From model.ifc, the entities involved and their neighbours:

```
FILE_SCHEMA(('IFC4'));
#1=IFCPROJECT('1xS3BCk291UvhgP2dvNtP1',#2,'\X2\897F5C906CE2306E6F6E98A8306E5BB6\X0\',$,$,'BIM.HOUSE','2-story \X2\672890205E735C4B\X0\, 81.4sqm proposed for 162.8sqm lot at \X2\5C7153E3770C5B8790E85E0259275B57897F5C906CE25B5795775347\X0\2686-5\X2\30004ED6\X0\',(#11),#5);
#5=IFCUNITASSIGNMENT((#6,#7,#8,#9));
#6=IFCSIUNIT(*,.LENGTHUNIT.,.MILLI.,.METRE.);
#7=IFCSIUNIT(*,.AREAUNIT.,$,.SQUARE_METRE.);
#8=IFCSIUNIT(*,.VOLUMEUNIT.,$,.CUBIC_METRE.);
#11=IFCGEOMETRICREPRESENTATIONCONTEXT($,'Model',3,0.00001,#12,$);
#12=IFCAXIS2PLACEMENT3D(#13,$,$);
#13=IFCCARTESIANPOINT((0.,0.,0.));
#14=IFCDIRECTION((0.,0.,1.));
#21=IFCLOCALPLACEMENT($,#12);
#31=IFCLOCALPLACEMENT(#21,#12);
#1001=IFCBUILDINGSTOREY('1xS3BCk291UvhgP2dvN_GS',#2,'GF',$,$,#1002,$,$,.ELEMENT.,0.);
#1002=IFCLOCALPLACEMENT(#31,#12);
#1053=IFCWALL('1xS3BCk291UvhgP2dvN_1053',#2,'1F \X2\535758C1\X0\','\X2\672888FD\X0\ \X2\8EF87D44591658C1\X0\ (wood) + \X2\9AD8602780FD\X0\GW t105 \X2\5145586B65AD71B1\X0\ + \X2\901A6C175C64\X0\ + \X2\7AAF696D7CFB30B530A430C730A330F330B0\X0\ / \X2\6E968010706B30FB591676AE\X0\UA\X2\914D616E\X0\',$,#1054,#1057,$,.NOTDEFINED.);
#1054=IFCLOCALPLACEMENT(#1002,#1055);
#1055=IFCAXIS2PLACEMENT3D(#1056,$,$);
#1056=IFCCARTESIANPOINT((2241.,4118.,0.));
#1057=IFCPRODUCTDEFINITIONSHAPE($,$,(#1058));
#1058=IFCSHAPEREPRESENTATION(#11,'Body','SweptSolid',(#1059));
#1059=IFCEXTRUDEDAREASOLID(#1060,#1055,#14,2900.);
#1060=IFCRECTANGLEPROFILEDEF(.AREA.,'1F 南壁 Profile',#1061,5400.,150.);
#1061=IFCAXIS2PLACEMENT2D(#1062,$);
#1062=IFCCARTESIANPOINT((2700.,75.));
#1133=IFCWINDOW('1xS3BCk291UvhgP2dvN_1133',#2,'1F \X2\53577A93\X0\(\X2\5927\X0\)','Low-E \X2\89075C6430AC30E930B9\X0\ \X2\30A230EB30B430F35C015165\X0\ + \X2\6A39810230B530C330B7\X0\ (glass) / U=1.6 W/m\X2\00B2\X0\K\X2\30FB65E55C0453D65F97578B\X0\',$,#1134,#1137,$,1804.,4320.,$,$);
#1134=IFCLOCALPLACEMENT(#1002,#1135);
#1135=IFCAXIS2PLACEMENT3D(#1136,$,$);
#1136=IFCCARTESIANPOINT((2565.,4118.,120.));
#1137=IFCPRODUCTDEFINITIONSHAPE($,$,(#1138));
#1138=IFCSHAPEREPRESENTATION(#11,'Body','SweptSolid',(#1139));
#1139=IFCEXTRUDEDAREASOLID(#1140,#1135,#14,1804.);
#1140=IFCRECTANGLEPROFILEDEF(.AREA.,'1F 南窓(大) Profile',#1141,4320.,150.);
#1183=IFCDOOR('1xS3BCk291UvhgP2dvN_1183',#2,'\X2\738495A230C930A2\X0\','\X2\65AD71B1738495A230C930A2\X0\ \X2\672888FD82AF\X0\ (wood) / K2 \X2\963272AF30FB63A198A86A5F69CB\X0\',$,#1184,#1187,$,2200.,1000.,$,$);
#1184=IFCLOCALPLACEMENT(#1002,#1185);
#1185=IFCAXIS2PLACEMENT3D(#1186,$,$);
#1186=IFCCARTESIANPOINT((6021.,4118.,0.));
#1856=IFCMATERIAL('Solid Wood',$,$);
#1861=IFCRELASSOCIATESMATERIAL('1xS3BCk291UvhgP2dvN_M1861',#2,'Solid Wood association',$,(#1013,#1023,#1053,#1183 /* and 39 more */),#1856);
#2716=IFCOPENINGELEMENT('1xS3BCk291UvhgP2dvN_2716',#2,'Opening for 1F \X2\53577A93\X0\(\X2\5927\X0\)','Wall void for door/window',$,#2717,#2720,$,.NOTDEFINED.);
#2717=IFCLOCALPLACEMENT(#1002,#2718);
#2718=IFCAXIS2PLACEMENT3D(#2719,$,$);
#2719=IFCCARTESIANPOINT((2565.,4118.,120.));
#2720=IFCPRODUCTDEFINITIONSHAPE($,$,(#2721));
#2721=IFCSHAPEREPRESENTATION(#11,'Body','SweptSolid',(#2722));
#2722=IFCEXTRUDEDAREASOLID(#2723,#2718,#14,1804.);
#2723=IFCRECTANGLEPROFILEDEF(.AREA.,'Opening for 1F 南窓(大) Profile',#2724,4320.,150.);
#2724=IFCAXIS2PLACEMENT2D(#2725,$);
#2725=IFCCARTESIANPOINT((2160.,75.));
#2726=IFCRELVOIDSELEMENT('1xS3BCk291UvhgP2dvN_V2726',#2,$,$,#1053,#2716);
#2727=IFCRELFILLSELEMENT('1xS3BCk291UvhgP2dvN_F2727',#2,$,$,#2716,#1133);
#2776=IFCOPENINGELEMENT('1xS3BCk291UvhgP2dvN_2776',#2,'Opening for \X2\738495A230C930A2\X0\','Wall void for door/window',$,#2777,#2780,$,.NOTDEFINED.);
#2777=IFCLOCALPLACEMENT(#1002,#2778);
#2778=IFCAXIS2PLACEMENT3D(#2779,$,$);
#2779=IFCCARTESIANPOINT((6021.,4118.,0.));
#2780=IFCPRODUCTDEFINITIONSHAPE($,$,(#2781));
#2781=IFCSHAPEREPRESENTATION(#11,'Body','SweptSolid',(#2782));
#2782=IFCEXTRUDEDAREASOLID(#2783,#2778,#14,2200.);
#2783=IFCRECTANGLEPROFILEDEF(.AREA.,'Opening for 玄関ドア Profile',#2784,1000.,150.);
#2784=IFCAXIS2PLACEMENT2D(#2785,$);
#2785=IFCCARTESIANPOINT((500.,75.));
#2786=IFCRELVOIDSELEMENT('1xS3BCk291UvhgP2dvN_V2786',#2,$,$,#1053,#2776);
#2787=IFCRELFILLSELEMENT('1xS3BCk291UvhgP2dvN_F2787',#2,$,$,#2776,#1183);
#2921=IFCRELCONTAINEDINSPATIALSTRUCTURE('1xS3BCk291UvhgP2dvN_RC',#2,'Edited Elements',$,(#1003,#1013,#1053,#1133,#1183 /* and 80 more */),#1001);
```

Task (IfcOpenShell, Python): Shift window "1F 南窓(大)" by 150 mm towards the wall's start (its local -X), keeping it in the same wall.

```python
import ifcopenshell
import ifcopenshell.api.geometry
import ifcopenshell.util.placement
import ifcopenshell.util.unit

model = ifcopenshell.open("model.ifc")
unit_scale = ifcopenshell.util.unit.calculate_unit_scale(model)

window = model.by_guid("1xS3BCk291UvhgP2dvN_1133")
opening = window.FillsVoids[0].RelatingOpeningElement
wall = opening.VoidsElements[0].RelatingBuildingElement

wall_matrix = ifcopenshell.util.placement.get_local_placement(wall.ObjectPlacement)
shift = wall_matrix[:3, 0] * -0.15 / unit_scale
before = ifcopenshell.util.placement.get_local_placement(window.ObjectPlacement)[:3, 3].copy()

# The window is not placed relative to its opening, so move both.
for product in (opening, window):
    matrix = ifcopenshell.util.placement.get_local_placement(product.ObjectPlacement)
    matrix[:3, 3] += shift
    ifcopenshell.api.geometry.edit_object_placement(model, product=product, matrix=matrix, is_si=False)

after = ifcopenshell.util.placement.get_local_placement(window.ObjectPlacement)[:3, 3]
print("window moved by", (after - before).round(3) + 0.0)

model.write("model-out.ifc")
```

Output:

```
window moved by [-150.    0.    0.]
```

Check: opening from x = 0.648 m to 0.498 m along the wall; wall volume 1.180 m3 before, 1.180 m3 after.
